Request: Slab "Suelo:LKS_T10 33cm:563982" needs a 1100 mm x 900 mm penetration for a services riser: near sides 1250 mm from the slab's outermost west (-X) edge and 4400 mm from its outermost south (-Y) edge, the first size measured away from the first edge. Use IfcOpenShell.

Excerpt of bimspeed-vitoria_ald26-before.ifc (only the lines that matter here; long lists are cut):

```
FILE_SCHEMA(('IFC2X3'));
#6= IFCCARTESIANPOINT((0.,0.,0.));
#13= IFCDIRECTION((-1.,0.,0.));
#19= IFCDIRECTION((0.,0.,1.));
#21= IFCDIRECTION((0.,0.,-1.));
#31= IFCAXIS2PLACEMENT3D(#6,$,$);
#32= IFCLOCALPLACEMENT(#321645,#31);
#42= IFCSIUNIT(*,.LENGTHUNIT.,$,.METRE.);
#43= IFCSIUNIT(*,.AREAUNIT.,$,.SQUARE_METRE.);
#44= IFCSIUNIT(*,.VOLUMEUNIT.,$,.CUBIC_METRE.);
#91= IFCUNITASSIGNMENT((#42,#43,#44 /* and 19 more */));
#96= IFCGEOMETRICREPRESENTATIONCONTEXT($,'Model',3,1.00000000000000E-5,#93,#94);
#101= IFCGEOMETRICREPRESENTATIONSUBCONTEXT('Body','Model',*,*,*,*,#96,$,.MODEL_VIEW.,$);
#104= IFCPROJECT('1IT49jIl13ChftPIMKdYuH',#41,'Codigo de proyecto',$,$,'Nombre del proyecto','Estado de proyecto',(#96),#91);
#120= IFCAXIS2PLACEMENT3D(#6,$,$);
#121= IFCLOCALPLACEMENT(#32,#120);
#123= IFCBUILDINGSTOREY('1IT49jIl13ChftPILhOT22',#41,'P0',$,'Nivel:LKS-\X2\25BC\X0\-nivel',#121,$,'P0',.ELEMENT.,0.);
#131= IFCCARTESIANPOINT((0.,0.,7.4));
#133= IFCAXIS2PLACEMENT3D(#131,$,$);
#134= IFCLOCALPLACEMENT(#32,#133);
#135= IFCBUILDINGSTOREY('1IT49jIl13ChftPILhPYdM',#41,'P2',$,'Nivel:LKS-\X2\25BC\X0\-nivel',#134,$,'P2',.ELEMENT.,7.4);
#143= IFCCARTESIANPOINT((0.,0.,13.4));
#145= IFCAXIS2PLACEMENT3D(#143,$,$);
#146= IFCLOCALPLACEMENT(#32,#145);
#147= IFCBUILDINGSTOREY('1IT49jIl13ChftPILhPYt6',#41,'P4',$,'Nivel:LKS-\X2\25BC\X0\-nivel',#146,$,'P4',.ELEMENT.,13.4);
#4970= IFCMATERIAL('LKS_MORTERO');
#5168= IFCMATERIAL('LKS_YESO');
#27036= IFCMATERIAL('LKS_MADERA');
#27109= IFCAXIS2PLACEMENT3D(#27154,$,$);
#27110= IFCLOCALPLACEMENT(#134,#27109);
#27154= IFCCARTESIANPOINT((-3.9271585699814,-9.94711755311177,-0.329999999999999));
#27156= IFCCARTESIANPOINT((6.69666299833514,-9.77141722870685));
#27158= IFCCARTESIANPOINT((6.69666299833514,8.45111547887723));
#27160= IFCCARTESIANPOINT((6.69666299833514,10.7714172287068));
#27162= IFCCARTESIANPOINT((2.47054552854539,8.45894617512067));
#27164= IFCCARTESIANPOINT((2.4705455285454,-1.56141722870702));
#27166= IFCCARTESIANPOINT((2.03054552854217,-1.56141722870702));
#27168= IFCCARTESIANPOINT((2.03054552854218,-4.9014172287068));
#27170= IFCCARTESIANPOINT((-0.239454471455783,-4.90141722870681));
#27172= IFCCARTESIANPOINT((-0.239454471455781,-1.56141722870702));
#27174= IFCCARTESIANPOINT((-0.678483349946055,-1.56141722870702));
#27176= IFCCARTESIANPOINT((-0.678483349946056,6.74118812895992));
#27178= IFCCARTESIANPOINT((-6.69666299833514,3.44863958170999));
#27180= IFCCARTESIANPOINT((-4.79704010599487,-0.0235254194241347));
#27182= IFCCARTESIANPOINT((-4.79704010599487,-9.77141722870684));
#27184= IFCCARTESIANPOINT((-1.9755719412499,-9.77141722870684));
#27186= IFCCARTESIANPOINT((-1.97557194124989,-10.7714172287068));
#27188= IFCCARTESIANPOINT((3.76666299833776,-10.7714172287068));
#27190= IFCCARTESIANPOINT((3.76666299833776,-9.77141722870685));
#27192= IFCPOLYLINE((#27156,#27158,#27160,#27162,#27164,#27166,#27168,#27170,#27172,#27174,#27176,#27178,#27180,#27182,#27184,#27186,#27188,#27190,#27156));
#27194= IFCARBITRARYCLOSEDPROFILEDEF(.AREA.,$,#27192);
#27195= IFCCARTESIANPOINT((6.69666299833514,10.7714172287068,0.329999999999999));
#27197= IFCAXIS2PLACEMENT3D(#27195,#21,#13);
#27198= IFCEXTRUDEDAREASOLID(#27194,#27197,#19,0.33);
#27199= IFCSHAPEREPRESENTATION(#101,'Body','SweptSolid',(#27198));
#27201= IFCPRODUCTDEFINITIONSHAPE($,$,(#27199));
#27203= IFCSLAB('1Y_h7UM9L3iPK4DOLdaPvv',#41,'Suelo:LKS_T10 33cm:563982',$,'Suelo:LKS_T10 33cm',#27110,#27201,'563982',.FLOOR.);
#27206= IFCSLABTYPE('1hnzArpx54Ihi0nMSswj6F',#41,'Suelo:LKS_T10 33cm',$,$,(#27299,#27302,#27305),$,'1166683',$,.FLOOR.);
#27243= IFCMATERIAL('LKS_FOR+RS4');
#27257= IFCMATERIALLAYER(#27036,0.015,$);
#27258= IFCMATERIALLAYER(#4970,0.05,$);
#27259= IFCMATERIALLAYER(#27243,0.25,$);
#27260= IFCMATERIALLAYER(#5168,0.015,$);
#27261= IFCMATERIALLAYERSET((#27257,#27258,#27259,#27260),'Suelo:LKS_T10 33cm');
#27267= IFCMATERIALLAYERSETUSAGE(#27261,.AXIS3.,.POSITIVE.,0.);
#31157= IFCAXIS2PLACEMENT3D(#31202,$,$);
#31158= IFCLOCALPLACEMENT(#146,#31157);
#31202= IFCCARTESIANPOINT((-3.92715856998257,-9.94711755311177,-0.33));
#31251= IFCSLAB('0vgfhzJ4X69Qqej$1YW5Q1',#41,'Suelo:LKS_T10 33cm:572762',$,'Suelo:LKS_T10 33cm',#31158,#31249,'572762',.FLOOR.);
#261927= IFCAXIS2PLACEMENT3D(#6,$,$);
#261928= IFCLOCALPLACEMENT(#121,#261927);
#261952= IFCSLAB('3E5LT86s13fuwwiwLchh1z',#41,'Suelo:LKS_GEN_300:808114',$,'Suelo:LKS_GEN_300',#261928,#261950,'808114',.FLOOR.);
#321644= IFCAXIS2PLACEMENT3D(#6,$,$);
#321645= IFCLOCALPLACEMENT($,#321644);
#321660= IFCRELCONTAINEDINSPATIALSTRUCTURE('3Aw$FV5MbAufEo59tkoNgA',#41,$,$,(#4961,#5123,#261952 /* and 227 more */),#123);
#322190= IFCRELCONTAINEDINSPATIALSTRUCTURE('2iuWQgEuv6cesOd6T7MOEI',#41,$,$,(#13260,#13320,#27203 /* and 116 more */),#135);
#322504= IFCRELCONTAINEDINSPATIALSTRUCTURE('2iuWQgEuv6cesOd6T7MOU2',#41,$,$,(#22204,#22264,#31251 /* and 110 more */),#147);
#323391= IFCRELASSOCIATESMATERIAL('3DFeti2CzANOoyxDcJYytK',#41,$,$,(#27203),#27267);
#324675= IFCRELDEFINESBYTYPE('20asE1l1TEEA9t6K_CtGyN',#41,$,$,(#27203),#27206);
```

```python
import numpy as np
import ifcopenshell
import ifcopenshell.api.feature
import ifcopenshell.api.geometry
import ifcopenshell.api.root
import ifcopenshell.geom
import ifcopenshell.util.placement
import ifcopenshell.util.representation
import ifcopenshell.util.shape
import ifcopenshell.util.unit

model = ifcopenshell.open("bimspeed-vitoria_ald26-before.ifc")
unit_scale = ifcopenshell.util.unit.calculate_unit_scale(model)
settings = ifcopenshell.geom.settings()


def volume(element):
    """Net volume in cubic metres, openings subtracted."""
    shape = ifcopenshell.geom.create_shape(settings, element)
    return ifcopenshell.util.shape.get_volume(shape.geometry)


slab = model.by_id(27203)
before = volume(slab)

# Extent in the slab's own axes, in metres. The edges named are its -X and -Y sides.
slab_shape = ifcopenshell.geom.create_shape(settings, slab)
vertices = ifcopenshell.util.shape.get_vertices(slab_shape.geometry)
x_min, y_min, bottom = vertices.min(axis=0)
top = vertices[:, 2].max()

opening = ifcopenshell.api.root.create_entity(model, ifc_class="IfcOpeningElement", name="Services riser opening")
context = ifcopenshell.util.representation.get_context(model, "Model", "Body", "MODEL_VIEW")
width, depth = 1.1, 0.9
outline = [(0.0, 0.0), (width, 0.0), (width, depth), (0.0, depth), (0.0, 0.0)]
# Overshoot both faces by 50 mm so the cut is clean.
shape = ifcopenshell.api.geometry.add_slab_representation(
    model, context=context, depth=top - bottom + 0.1, polyline=outline
)
ifcopenshell.api.geometry.assign_representation(model, product=opening, representation=shape)

matrix = ifcopenshell.util.placement.get_local_placement(slab.ObjectPlacement)
matrix[:, 3] = matrix @ np.append(np.array([x_min + 1.25, y_min + 4.4, bottom - 0.05]) / unit_scale, 1.0)
ifcopenshell.api.geometry.edit_object_placement(model, product=opening, matrix=matrix, is_si=False)
ifcopenshell.api.feature.add_feature(model, feature=opening, element=slab)

after = volume(slab)

print(f"slab volume {before:.3f} -> {after:.3f} m3")

model.write("bimspeed-vitoria_ald26-before-out.ifc")
```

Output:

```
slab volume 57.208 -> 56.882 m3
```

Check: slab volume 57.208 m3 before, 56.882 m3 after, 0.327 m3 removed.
